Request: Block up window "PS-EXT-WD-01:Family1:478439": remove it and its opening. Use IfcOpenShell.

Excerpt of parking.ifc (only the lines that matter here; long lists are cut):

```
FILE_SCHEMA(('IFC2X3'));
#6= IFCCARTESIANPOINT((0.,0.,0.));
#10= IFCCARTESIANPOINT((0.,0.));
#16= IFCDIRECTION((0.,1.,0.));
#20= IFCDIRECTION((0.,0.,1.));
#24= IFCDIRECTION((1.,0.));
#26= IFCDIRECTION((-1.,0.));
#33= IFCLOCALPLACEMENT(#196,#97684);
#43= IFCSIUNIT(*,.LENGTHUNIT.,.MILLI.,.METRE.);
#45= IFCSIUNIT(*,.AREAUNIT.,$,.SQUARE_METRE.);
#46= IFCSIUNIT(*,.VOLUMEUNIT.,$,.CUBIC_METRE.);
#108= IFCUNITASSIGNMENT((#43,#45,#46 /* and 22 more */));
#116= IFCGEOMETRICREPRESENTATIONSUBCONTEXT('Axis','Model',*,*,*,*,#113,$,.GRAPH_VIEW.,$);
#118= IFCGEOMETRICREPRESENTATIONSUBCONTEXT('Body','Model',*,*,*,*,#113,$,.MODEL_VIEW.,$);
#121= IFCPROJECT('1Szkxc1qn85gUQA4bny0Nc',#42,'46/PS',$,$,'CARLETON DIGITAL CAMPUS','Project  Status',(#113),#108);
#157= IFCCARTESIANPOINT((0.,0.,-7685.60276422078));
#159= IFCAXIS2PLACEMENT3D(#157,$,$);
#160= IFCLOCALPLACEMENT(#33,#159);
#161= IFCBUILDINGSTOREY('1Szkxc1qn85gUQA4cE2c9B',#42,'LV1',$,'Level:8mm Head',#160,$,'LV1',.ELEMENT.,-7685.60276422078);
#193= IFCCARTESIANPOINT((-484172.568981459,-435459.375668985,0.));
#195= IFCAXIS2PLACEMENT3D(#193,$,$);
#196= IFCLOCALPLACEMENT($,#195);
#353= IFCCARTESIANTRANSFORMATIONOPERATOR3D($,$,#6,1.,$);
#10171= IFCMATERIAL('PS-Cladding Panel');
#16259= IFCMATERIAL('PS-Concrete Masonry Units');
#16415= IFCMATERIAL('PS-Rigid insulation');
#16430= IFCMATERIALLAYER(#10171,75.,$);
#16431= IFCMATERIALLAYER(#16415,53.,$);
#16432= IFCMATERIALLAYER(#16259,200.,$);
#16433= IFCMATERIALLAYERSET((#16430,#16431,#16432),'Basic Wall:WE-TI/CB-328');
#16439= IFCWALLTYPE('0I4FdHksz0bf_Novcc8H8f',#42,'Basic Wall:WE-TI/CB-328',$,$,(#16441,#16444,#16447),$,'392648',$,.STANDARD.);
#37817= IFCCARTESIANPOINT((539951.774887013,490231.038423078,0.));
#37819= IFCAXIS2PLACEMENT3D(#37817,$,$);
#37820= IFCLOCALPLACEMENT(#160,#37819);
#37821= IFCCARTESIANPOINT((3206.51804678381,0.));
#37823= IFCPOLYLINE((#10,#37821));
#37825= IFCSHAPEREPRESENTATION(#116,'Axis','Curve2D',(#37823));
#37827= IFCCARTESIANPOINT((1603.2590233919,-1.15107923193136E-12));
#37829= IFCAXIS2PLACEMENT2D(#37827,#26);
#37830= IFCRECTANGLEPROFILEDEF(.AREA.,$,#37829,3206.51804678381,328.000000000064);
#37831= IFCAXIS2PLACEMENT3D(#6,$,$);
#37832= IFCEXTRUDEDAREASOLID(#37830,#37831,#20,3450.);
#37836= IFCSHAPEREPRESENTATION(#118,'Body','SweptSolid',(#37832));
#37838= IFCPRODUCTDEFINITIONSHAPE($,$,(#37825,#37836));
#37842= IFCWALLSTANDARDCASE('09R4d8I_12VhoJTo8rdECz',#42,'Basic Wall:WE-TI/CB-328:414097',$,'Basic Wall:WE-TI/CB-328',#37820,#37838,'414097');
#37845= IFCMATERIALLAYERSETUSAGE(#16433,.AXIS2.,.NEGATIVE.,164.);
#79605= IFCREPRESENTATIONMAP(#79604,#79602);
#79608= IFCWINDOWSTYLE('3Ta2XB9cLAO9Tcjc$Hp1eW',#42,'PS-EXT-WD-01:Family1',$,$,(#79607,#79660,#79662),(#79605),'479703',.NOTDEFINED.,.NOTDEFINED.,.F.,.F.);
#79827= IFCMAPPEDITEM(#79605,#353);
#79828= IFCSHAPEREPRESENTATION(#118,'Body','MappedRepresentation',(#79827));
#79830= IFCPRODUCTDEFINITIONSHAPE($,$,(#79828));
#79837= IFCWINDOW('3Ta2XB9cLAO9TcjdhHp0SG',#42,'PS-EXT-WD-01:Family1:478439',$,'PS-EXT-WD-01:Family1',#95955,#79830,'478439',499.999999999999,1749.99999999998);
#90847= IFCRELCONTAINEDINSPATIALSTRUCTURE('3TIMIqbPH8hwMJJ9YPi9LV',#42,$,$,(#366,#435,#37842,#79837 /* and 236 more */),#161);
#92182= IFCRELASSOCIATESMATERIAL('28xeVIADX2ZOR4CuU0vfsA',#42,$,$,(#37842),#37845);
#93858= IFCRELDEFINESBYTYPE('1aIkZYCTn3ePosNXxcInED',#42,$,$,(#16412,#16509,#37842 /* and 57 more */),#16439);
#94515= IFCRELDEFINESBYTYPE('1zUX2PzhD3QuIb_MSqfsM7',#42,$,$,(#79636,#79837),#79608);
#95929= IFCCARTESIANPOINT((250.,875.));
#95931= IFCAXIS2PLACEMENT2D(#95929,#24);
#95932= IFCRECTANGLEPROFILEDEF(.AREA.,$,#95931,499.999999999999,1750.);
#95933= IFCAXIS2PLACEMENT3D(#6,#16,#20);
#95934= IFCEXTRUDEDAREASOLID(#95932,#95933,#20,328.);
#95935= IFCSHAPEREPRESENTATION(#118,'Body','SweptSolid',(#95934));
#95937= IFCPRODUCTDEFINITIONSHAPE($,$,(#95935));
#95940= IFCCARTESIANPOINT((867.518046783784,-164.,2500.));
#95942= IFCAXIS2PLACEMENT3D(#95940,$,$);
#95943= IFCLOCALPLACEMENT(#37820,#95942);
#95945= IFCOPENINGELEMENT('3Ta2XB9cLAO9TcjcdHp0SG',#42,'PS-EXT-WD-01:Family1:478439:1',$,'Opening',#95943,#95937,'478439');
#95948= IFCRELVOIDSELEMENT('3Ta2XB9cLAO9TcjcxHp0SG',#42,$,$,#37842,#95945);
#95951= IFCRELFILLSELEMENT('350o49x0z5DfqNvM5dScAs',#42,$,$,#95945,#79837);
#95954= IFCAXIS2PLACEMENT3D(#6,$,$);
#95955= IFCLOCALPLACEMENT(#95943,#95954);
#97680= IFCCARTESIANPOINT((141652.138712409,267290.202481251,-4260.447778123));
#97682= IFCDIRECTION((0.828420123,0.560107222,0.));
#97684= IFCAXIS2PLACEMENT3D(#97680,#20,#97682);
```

```python
import ifcopenshell
import ifcopenshell.api.feature
import ifcopenshell.api.root
import ifcopenshell.geom
import ifcopenshell.util.shape

model = ifcopenshell.open("parking.ifc")
settings = ifcopenshell.geom.settings()


def volume(element):
    """Net volume in cubic metres, openings subtracted."""
    shape = ifcopenshell.geom.create_shape(settings, element)
    return ifcopenshell.util.shape.get_volume(shape.geometry)


window = model.by_id(79837)
opening = window.FillsVoids[0].RelatingOpeningElement
wall = opening.VoidsElements[0].RelatingBuildingElement
before = volume(wall)

ifcopenshell.api.root.remove_product(model, product=window)
ifcopenshell.api.feature.remove_feature(model, feature=opening)

after = volume(wall)

print(f"wall volume {before:.3f} -> {after:.3f} m3")

model.write("parking_v2.ifc")
```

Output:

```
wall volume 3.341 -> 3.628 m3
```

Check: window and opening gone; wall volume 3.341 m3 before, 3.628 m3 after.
